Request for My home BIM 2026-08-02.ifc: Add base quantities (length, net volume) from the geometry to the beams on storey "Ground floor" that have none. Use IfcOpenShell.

First a look at what the model holds.

```python
import ifcopenshell
import ifcopenshell.util.element
import ifcopenshell.util.unit

model = ifcopenshell.open("My home BIM 2026-08-02.ifc")
print(model.schema)
for unit_type in ("LENGTHUNIT", "AREAUNIT", "VOLUMEUNIT"):
    print(unit_type, ifcopenshell.util.unit.calculate_unit_scale(model, unit_type))
storey = next(s for s in model.by_type("IfcBuildingStorey") if s.Name == "Ground floor")
beams = [e for e in ifcopenshell.util.element.get_decomposition(storey) if e.is_a("IfcBeam")]
for e in sorted(beams, key=lambda e: e.id()):
    print(e.id(), e.is_a(), e.Name, list(ifcopenshell.util.element.get_psets(e, qtos_only=True)), sep=" | ")
```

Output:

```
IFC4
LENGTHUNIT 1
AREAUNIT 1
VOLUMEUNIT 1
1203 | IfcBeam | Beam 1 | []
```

```python
import ifcopenshell
import ifcopenshell.api.pset
import ifcopenshell.geom
import ifcopenshell.util.element
import ifcopenshell.util.shape
import ifcopenshell.util.unit

model = ifcopenshell.open("My home BIM 2026-08-02.ifc")
unit_scale = ifcopenshell.util.unit.calculate_unit_scale(model)
volume_scale = ifcopenshell.util.unit.calculate_unit_scale(model, "VOLUMEUNIT")
settings = ifcopenshell.geom.settings()

storey = next(s for s in model.by_type("IfcBuildingStorey") if s.Name == "Ground floor")
beams = [e for e in ifcopenshell.util.element.get_decomposition(storey) if e.is_a("IfcBeam")]

for e in sorted(beams, key=lambda e: e.id()):
    if ifcopenshell.util.element.get_psets(e, qtos_only=True, should_inherit=False):
        continue
    # Geometry comes back in metres, in the element's own axes.
    shape = ifcopenshell.geom.create_shape(settings, e)
    values = {
        "Length": ifcopenshell.util.shape.get_max_xyz(shape.geometry) / unit_scale,
        "NetVolume": ifcopenshell.util.shape.get_volume(shape.geometry) / volume_scale,
    }
    qto = ifcopenshell.api.pset.add_qto(model, product=e, name="Qto_BeamBaseQuantities")
    ifcopenshell.api.pset.edit_qto(model, qto=qto, properties=values)
    print(e.id(), {k: round(v, 3) for k, v in values.items()})

model.write("My home BIM 2026-08-02_edited.ifc")
```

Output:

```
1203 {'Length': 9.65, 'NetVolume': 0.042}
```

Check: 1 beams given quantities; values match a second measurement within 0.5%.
